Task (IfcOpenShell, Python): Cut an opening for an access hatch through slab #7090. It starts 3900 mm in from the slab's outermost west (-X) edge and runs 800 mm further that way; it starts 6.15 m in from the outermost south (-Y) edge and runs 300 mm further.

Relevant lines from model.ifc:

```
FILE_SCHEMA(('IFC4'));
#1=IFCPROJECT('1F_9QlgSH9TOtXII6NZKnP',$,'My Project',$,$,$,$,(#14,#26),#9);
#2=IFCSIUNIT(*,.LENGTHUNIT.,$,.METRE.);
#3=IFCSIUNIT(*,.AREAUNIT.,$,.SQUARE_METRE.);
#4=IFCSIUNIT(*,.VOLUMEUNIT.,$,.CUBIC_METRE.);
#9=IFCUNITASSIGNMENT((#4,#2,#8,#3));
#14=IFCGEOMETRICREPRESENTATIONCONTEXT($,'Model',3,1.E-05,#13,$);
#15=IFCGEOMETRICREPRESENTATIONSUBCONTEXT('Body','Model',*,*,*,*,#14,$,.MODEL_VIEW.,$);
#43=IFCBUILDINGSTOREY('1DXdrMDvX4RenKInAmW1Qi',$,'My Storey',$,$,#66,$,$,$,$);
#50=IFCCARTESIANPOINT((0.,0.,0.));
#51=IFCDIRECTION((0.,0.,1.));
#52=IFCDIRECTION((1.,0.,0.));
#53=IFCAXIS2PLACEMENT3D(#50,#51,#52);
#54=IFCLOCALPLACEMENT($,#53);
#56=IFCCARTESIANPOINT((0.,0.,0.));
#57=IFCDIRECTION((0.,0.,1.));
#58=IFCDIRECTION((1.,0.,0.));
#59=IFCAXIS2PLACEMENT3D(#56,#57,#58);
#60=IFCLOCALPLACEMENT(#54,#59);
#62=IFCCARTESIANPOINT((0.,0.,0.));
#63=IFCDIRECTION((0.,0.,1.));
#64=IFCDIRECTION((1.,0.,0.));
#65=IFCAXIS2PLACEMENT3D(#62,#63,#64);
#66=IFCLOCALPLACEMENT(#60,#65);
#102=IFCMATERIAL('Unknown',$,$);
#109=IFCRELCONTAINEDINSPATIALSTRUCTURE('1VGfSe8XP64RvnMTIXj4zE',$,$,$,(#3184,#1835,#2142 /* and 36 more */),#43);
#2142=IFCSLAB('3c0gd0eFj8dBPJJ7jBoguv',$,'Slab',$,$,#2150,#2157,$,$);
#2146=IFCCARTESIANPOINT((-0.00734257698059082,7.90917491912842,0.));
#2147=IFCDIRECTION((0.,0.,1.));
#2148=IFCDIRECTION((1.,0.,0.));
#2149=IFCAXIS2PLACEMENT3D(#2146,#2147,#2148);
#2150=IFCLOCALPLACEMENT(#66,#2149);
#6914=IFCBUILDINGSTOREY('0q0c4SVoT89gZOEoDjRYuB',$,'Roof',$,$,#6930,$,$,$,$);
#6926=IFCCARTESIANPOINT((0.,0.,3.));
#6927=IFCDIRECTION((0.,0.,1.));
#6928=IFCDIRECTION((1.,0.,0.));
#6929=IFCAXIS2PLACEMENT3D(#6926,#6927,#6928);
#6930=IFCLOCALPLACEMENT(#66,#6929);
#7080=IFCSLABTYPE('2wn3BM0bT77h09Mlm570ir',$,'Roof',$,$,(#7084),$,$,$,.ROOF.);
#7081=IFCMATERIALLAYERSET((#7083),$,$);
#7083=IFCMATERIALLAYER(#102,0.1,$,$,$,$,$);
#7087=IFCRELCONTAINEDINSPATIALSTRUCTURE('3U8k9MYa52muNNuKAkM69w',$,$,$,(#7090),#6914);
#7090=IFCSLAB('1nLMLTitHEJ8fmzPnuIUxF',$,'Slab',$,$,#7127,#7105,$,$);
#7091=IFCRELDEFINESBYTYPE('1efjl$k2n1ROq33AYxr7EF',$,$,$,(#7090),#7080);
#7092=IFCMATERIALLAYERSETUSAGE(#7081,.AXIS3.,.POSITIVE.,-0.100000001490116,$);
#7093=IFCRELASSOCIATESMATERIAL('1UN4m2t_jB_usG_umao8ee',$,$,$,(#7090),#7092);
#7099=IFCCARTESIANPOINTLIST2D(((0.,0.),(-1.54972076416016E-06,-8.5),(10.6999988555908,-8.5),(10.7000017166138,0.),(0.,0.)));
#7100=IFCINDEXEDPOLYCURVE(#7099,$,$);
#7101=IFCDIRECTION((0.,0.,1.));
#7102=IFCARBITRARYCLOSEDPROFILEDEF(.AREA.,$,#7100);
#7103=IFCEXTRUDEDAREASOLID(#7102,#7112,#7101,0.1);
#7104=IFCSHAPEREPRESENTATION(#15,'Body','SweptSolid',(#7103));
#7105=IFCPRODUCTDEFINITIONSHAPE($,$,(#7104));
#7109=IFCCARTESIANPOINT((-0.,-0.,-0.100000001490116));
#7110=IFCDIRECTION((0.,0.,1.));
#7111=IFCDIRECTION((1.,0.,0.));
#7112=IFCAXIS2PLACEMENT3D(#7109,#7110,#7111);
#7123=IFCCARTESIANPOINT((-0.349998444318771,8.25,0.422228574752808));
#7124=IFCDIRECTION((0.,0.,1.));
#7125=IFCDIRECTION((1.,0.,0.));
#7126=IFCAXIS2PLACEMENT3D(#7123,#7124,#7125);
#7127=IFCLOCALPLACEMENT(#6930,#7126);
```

```python
import numpy as np
import ifcopenshell
import ifcopenshell.api.feature
import ifcopenshell.api.geometry
import ifcopenshell.api.root
import ifcopenshell.geom
import ifcopenshell.util.placement
import ifcopenshell.util.representation
import ifcopenshell.util.shape
import ifcopenshell.util.unit

model = ifcopenshell.open("model.ifc")
unit_scale = ifcopenshell.util.unit.calculate_unit_scale(model)
settings = ifcopenshell.geom.settings()


def volume(element):
    """Net volume in cubic metres, openings subtracted."""
    shape = ifcopenshell.geom.create_shape(settings, element)
    return ifcopenshell.util.shape.get_volume(shape.geometry)


slab = model.by_guid("1nLMLTitHEJ8fmzPnuIUxF")
before = volume(slab)

# Extent in the slab's own axes, in metres. The edges named are its -X and -Y sides.
slab_shape = ifcopenshell.geom.create_shape(settings, slab)
vertices = ifcopenshell.util.shape.get_vertices(slab_shape.geometry)
x_min, y_min, bottom = vertices.min(axis=0)
top = vertices[:, 2].max()

opening = ifcopenshell.api.root.create_entity(model, ifc_class="IfcOpeningElement", name="Access hatch opening", predefined_type="OPENING")
context = ifcopenshell.util.representation.get_context(model, "Model", "Body", "MODEL_VIEW")
width, depth = 0.8, 0.3
outline = [(0.0, 0.0), (width, 0.0), (width, depth), (0.0, depth), (0.0, 0.0)]
# Overshoot both faces by 50 mm so the cut is clean.
shape = ifcopenshell.api.geometry.add_slab_representation(
    model, context=context, depth=top - bottom + 0.1, polyline=outline
)
ifcopenshell.api.geometry.assign_representation(model, product=opening, representation=shape)

matrix = ifcopenshell.util.placement.get_local_placement(slab.ObjectPlacement)
matrix[:, 3] = matrix @ np.append(np.array([x_min + 3.9, y_min + 6.15, bottom - 0.05]) / unit_scale, 1.0)
ifcopenshell.api.geometry.edit_object_placement(model, product=opening, matrix=matrix, is_si=False)
ifcopenshell.api.feature.add_feature(model, feature=opening, element=slab)

after = volume(slab)

print(f"slab volume {before:.3f} -> {after:.3f} m3")

model.write("model_updated.ifc")
```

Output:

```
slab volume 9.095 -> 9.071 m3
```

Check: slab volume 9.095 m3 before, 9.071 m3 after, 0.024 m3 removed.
